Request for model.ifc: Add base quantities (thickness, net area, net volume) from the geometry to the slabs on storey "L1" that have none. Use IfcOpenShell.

First a look at what the model holds.

```python
import ifcopenshell
import ifcopenshell.util.element
import ifcopenshell.util.unit

model = ifcopenshell.open("model.ifc")
print(model.schema)
for unit_type in ("LENGTHUNIT", "AREAUNIT", "VOLUMEUNIT"):
    print(unit_type, ifcopenshell.util.unit.calculate_unit_scale(model, unit_type))
storey = next(s for s in model.by_type("IfcBuildingStorey") if s.Name == "L1")
slabs = [e for e in ifcopenshell.util.element.get_decomposition(storey) if e.is_a("IfcSlab")]
for e in sorted(slabs, key=lambda e: e.id()):
    print(e.id(), e.is_a(), e.Name, list(ifcopenshell.util.element.get_psets(e, qtos_only=True)), sep=" | ")
```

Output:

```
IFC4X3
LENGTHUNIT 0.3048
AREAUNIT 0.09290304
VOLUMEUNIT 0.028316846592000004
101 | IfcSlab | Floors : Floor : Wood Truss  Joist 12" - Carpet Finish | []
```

```python
import ifcopenshell
import ifcopenshell.api.pset
import ifcopenshell.geom
import ifcopenshell.util.element
import ifcopenshell.util.shape
import ifcopenshell.util.unit

model = ifcopenshell.open("model.ifc")
unit_scale = ifcopenshell.util.unit.calculate_unit_scale(model)
area_scale = ifcopenshell.util.unit.calculate_unit_scale(model, "AREAUNIT")
volume_scale = ifcopenshell.util.unit.calculate_unit_scale(model, "VOLUMEUNIT")
settings = ifcopenshell.geom.settings()

storey = next(s for s in model.by_type("IfcBuildingStorey") if s.Name == "L1")
slabs = [e for e in ifcopenshell.util.element.get_decomposition(storey) if e.is_a("IfcSlab")]

for e in sorted(slabs, key=lambda e: e.id()):
    if ifcopenshell.util.element.get_psets(e, qtos_only=True, should_inherit=False):
        continue
    # Geometry comes back in metres, in the element's own axes.
    shape = ifcopenshell.geom.create_shape(settings, e)
    values = {
        "Width": ifcopenshell.util.shape.get_z(shape.geometry) / unit_scale,
        "NetArea": ifcopenshell.util.shape.get_footprint_area(shape.geometry) / area_scale,
        "NetVolume": ifcopenshell.util.shape.get_volume(shape.geometry) / volume_scale,
    }
    qto = ifcopenshell.api.pset.add_qto(model, product=e, name="Qto_SlabBaseQuantities")
    ifcopenshell.api.pset.edit_qto(model, qto=qto, properties=values)
    print(e.id(), {k: round(v, 3) for k, v in values.items()})

model.write("model_edited.ifc")
```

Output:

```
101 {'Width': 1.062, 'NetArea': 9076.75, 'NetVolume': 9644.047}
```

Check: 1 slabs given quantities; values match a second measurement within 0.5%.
